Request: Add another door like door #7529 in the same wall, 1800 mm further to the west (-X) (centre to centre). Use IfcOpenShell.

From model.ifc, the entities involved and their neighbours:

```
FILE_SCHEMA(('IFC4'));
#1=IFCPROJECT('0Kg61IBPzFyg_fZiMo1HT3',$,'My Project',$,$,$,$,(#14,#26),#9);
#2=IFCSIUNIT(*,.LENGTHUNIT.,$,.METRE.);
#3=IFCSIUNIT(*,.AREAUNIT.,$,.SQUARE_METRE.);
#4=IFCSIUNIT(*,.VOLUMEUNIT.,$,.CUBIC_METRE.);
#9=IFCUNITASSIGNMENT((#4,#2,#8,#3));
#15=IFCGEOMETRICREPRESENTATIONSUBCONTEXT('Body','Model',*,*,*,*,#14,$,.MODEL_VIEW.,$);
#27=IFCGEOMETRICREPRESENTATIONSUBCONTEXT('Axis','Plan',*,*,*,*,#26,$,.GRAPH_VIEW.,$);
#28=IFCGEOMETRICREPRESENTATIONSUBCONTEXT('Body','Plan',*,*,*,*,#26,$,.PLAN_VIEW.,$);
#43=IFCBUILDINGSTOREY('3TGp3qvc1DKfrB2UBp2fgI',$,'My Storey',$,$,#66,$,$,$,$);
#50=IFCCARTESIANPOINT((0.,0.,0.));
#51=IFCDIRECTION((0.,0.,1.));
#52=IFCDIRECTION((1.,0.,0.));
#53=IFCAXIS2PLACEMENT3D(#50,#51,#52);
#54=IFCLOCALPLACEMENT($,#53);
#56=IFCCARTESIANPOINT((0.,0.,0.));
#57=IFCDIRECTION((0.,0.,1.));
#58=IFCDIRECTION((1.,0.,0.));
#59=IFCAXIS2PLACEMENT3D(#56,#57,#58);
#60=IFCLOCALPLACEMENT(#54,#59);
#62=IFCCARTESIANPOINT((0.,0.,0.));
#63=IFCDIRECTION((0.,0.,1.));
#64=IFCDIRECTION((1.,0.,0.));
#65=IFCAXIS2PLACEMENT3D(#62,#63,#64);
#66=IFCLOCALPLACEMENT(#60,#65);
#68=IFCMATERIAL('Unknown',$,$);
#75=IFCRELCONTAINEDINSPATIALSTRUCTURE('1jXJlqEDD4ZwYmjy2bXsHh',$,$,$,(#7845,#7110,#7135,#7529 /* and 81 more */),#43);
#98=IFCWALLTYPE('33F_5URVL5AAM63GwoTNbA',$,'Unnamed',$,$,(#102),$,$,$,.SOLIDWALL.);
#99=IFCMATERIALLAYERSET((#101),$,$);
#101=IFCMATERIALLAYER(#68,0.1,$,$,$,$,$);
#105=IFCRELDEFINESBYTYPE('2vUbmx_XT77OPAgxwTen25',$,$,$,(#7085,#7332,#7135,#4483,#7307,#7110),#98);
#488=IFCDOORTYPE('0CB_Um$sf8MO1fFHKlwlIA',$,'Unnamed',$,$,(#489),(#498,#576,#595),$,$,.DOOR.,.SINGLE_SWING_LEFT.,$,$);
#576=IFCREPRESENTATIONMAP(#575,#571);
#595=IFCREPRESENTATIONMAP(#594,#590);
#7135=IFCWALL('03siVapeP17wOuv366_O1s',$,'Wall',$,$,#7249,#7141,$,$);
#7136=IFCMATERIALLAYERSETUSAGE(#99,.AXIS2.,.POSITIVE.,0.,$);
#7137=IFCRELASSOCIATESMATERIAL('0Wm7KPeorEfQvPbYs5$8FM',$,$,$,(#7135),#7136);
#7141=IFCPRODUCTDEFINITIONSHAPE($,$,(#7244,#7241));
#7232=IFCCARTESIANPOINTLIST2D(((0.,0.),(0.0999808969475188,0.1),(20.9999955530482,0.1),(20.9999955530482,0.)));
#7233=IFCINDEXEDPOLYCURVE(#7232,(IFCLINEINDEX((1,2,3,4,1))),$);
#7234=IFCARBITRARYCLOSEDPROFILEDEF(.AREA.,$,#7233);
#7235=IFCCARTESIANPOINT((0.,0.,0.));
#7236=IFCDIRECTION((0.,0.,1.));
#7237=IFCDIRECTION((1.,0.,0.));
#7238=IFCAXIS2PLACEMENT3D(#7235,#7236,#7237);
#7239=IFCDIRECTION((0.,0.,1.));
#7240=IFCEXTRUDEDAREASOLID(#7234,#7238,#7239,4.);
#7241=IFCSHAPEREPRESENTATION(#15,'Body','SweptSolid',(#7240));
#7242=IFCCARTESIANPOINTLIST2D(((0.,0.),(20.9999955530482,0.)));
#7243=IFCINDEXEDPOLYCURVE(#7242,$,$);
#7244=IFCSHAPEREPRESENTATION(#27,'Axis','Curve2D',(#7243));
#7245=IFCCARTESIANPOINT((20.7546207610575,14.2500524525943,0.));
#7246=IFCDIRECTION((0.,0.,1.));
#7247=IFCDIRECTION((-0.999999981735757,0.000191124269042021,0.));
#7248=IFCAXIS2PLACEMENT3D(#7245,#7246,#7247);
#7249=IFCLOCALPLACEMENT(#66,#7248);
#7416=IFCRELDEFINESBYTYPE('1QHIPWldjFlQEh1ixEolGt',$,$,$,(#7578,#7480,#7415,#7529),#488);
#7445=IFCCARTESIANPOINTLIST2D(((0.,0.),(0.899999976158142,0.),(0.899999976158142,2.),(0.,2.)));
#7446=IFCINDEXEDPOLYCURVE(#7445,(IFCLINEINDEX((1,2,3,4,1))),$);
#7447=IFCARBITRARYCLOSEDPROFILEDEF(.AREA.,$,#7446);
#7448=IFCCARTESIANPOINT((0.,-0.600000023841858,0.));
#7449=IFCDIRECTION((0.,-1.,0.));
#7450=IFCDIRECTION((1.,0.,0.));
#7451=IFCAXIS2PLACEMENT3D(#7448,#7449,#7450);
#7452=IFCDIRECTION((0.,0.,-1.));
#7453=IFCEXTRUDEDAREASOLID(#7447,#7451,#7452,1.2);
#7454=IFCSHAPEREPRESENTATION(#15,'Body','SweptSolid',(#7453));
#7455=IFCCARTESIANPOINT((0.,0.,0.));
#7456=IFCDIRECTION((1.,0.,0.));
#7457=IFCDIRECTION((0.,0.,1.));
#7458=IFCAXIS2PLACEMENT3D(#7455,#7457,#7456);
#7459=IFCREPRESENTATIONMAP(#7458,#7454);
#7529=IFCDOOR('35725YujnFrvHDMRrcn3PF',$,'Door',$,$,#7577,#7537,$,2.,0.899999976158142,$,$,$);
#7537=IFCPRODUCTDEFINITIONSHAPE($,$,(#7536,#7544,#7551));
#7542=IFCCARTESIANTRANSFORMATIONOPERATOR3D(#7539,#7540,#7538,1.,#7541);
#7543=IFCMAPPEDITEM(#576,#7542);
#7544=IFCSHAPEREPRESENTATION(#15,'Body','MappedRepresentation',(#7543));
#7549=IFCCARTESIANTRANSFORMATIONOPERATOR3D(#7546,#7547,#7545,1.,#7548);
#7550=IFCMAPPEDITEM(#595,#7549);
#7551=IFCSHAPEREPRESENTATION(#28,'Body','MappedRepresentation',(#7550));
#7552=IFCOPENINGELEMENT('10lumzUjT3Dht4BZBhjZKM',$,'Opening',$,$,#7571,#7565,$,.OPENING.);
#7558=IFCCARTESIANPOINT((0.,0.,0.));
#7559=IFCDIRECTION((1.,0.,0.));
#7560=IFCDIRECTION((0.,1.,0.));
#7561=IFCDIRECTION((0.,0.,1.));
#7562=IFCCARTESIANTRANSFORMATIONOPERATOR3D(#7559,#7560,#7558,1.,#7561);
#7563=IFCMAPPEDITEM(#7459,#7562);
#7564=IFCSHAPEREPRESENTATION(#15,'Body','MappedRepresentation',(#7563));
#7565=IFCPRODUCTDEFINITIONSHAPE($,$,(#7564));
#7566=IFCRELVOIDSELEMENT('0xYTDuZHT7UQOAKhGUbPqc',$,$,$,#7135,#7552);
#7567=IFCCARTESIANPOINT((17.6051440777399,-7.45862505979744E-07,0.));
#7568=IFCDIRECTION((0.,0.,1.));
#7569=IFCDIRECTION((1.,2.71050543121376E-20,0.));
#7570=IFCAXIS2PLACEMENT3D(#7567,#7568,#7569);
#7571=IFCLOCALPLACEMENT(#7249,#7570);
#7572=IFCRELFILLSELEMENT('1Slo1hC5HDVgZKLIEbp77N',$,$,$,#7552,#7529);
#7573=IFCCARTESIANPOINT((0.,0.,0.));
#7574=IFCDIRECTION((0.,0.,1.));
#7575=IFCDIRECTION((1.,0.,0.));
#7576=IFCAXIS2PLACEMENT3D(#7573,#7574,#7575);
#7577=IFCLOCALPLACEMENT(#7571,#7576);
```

```python
import ifcopenshell
import ifcopenshell.api.feature
import ifcopenshell.api.geometry
import ifcopenshell.api.root
import ifcopenshell.geom
import ifcopenshell.util.element
import ifcopenshell.util.placement
import ifcopenshell.util.shape

model = ifcopenshell.open("model.ifc")
settings = ifcopenshell.geom.settings()


def volume(element):
    """Net volume in cubic metres, openings subtracted."""
    shape = ifcopenshell.geom.create_shape(settings, element)
    return ifcopenshell.util.shape.get_volume(shape.geometry)


door = model.by_guid("35725YujnFrvHDMRrcn3PF")
opening = door.FillsVoids[0].RelatingOpeningElement
wall = opening.VoidsElements[0].RelatingBuildingElement
before = volume(wall)
shift = ifcopenshell.util.placement.get_local_placement(wall.ObjectPlacement)[:3, 0] * 1.8

# copy_class copies the void relationship, type, container and properties, but no geometry.
new_opening = ifcopenshell.api.root.copy_class(model, product=opening)
new_opening.Representation = ifcopenshell.util.element.copy_deep(
    model, opening.Representation, exclude=["IfcGeometricRepresentationContext", "IfcRepresentationMap"]
)
new_door = ifcopenshell.api.root.copy_class(model, product=door)
new_door.Representation = ifcopenshell.util.element.copy_deep(
    model, door.Representation, exclude=["IfcGeometricRepresentationContext", "IfcRepresentationMap"]
)
ifcopenshell.api.feature.add_filling(model, opening=new_opening, element=new_door)

for old, new in ((opening, new_opening), (door, new_door)):
    matrix = ifcopenshell.util.placement.get_local_placement(old.ObjectPlacement)
    matrix[:3, 3] += shift
    ifcopenshell.api.geometry.edit_object_placement(model, product=new, matrix=matrix, is_si=False)

after = volume(wall)

print(f"wall volume {before:.3f} -> {after:.3f} m3")

model.write("model_v2.ifc")
```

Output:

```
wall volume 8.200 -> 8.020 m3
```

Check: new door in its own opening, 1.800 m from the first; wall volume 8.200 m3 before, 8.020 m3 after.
